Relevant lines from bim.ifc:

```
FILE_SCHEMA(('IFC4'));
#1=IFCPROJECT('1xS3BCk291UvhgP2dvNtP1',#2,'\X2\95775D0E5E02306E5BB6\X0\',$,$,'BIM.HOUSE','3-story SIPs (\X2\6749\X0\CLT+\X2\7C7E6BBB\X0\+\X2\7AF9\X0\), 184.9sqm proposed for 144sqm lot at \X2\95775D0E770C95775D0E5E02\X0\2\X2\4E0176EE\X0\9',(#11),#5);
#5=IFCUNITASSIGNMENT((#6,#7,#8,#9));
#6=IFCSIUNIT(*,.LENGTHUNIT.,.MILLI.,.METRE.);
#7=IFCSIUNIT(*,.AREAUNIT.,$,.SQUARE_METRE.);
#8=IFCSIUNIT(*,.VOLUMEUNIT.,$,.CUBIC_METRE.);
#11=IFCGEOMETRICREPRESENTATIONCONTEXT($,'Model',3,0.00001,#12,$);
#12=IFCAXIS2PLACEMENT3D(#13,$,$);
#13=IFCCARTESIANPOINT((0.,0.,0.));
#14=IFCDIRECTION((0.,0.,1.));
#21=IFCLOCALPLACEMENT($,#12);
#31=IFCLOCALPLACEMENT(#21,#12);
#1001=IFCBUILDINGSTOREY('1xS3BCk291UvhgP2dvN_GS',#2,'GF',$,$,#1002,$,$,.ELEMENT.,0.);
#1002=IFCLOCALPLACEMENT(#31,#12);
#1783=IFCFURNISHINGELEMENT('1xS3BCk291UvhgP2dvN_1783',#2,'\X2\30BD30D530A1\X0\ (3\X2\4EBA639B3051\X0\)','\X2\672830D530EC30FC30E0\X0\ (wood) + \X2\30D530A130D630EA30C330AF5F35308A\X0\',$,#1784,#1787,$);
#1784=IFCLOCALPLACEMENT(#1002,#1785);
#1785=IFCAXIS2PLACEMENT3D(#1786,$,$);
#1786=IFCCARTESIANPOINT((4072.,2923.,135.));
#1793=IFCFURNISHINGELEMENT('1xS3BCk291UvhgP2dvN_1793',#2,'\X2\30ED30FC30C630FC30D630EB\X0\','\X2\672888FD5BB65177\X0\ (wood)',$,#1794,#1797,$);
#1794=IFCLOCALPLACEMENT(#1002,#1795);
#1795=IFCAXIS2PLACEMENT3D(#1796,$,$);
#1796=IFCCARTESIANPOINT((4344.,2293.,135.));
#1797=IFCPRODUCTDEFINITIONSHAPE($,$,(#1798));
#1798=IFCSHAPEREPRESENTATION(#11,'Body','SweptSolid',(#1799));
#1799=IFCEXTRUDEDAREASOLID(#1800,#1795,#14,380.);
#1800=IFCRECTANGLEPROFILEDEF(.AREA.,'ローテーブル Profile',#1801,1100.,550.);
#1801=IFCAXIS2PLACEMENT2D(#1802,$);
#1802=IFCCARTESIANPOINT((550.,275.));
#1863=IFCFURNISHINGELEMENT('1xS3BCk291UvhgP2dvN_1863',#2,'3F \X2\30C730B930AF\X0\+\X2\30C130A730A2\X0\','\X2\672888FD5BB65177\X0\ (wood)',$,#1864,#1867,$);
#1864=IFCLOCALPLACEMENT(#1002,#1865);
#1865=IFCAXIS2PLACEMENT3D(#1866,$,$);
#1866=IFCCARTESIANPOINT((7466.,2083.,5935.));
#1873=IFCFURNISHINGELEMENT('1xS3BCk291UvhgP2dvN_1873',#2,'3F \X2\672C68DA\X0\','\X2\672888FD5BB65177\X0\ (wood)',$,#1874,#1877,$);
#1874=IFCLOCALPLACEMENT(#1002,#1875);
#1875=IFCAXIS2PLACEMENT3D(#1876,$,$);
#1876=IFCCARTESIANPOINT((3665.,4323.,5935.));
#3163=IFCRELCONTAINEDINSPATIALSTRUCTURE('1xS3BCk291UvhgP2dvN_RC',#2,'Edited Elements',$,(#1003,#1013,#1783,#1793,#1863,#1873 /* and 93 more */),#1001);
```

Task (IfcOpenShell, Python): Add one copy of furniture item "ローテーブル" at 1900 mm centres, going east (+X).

```python
import numpy as np
import ifcopenshell
import ifcopenshell.api.geometry
import ifcopenshell.api.root
import ifcopenshell.util.element
import ifcopenshell.util.placement
import ifcopenshell.util.unit

model = ifcopenshell.open("bim.ifc")
unit_scale = ifcopenshell.util.unit.calculate_unit_scale(model)


def reuse_history(source, copy):
    """copy_class also copies each property set's owner history, people and application; keep the originals."""
    for rel in copy.IsDefinedBy:
        if rel.is_a("IfcRelDefinesByProperties") and (history := rel.RelatingPropertyDefinition.OwnerHistory):
            rel.RelatingPropertyDefinition.OwnerHistory = source.OwnerHistory
            ifcopenshell.util.element.remove_deep2(model, history)


source = model.by_guid("1xS3BCk291UvhgP2dvN_1793")
base = ifcopenshell.util.placement.get_local_placement(source.ObjectPlacement)
step = np.array([1.0, 0.0, 0.0]) * 1.9 / unit_scale

for i in range(1, 2):
    copy = ifcopenshell.api.root.copy_class(model, product=source)
    copy.Representation = ifcopenshell.util.element.copy_deep(
        model, source.Representation, exclude=["IfcGeometricRepresentationContext", "IfcRepresentationMap"]
    )
    reuse_history(source, copy)
    matrix = base.copy()
    matrix[:3, 3] += i * step
    print("added at", matrix[:3, 3].round(3) + 0.0)
    ifcopenshell.api.geometry.edit_object_placement(model, product=copy, matrix=matrix, is_si=False)

model.write("bim_v2.ifc")
```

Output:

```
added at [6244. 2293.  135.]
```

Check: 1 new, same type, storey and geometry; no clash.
